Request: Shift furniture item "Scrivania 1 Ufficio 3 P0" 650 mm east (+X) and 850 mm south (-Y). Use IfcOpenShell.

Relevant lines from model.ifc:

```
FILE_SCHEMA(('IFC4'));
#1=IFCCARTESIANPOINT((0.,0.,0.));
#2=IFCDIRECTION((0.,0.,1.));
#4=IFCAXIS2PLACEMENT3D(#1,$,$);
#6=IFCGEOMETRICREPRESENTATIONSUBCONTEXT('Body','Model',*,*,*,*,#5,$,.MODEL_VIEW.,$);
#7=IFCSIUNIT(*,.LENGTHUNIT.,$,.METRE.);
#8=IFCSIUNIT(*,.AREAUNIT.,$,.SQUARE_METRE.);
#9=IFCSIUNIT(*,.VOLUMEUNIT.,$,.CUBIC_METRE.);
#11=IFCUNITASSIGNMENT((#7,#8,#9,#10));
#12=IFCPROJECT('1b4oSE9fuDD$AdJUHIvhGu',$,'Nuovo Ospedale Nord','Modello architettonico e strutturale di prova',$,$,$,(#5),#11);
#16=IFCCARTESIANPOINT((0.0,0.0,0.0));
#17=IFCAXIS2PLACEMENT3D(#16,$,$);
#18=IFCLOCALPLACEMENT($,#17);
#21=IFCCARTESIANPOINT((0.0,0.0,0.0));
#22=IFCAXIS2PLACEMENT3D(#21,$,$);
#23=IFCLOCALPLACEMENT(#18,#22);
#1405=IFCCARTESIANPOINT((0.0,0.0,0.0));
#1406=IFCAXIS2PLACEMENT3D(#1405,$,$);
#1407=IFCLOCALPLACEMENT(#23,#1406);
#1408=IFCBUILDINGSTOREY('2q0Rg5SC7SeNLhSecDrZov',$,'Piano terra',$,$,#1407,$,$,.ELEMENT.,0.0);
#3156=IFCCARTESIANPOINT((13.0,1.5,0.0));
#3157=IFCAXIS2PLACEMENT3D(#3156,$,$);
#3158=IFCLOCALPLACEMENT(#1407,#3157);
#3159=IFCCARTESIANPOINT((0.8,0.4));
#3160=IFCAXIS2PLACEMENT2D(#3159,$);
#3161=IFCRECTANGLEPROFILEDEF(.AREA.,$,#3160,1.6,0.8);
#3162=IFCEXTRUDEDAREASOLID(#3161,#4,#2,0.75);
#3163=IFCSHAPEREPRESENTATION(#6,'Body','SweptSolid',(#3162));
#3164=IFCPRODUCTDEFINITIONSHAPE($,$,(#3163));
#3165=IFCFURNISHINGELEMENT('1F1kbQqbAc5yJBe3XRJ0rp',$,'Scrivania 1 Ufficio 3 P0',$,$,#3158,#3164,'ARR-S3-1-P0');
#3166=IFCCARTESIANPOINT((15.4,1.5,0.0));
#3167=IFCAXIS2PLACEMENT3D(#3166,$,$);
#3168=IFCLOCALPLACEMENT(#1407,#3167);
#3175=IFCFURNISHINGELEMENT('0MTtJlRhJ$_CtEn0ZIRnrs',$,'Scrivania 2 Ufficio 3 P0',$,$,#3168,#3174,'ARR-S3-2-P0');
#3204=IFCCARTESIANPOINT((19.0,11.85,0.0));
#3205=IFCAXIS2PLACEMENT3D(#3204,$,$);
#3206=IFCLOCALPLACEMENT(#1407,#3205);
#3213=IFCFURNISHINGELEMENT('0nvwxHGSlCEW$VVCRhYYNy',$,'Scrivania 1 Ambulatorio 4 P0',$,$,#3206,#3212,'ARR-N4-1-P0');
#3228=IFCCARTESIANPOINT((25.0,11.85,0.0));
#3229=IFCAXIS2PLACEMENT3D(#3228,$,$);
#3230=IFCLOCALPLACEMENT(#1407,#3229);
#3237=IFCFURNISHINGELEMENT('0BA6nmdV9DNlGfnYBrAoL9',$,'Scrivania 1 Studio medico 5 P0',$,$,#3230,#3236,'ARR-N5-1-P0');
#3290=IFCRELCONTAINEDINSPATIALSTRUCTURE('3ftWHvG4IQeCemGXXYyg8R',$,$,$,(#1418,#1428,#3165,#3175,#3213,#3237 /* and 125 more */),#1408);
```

```python
import ifcopenshell
import ifcopenshell.api.geometry
import ifcopenshell.util.placement
import ifcopenshell.util.unit

model = ifcopenshell.open("model.ifc")
unit_scale = ifcopenshell.util.unit.calculate_unit_scale(model)

item = model.by_id(3165)
matrix = ifcopenshell.util.placement.get_local_placement(item.ObjectPlacement)
matrix[0, 3] += 0.65 / unit_scale
matrix[1, 3] -= 0.85 / unit_scale
ifcopenshell.api.geometry.edit_object_placement(model, product=item, matrix=matrix, is_si=False)

print(ifcopenshell.util.placement.get_local_placement(item.ObjectPlacement).round(3) + 0.0)

model.write("model_updated.ifc")
```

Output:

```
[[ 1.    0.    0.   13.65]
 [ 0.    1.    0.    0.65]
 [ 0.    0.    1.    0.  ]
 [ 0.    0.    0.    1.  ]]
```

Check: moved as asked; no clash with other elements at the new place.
